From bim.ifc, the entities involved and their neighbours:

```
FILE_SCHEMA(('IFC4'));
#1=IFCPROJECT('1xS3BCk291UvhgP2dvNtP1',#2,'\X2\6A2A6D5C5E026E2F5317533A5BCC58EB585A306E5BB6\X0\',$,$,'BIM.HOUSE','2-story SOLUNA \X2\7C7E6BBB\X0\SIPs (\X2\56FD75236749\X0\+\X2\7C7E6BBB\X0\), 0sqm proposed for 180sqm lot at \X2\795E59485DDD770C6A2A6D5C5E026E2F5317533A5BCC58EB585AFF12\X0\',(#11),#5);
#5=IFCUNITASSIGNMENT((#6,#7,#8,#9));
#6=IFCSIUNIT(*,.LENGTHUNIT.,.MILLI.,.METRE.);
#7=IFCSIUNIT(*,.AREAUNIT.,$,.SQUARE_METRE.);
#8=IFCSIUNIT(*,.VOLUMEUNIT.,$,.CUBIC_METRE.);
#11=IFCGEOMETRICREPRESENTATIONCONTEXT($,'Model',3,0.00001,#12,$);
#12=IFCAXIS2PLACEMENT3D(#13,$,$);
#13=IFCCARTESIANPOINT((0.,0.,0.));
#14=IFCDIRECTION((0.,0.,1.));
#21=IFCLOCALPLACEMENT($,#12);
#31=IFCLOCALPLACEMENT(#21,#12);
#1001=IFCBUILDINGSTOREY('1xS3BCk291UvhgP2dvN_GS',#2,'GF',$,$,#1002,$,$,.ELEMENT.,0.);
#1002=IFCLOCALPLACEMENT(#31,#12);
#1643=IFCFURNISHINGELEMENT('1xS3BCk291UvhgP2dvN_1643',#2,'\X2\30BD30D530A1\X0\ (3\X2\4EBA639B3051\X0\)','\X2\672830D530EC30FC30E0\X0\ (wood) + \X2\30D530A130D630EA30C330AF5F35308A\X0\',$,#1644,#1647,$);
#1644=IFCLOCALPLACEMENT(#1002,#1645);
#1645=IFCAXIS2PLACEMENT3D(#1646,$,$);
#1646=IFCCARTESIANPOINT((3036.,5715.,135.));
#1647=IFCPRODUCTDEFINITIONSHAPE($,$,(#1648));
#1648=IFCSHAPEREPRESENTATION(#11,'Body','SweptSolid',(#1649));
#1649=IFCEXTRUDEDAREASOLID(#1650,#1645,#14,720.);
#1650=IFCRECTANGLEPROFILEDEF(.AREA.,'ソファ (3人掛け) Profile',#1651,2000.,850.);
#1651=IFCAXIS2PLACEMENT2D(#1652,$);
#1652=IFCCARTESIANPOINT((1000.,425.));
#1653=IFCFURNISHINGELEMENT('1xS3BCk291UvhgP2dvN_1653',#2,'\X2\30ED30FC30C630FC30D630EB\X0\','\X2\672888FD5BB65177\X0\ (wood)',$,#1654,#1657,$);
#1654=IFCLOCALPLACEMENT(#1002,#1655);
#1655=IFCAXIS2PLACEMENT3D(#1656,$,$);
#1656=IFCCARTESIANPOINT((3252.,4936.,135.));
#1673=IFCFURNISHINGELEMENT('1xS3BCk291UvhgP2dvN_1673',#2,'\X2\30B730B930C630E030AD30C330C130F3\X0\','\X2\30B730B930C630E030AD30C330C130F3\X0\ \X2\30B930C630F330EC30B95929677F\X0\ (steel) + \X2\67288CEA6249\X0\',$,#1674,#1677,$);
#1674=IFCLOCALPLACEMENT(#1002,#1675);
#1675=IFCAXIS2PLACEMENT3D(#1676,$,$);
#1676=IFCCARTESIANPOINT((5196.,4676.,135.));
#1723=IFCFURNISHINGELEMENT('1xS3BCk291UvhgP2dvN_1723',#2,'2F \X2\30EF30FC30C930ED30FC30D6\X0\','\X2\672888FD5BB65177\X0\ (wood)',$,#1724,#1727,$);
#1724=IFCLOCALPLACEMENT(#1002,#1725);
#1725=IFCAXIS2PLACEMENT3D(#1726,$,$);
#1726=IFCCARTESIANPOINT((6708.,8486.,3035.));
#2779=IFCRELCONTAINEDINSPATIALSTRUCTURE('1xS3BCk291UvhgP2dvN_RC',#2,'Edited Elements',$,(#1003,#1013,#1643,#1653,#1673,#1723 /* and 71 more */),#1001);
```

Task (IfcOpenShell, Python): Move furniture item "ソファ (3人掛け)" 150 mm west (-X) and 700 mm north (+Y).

```python
import ifcopenshell
import ifcopenshell.api.geometry
import ifcopenshell.util.placement

model = ifcopenshell.open("bim.ifc")

item = model.by_id(1643)
matrix = ifcopenshell.util.placement.get_local_placement(item.ObjectPlacement)
matrix[0, 3] -= 150.0
matrix[1, 3] += 700.0
ifcopenshell.api.geometry.edit_object_placement(model, product=item, matrix=matrix, is_si=False)

print(ifcopenshell.util.placement.get_local_placement(item.ObjectPlacement).round(3) + 0.0)

model.write("bim-out.ifc")
```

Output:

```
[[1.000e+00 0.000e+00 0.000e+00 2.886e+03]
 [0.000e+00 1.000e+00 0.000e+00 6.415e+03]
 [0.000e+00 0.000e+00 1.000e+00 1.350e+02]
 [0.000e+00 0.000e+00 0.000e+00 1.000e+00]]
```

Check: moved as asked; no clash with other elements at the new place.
